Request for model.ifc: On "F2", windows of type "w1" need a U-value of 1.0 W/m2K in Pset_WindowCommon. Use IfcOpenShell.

First a look at what the model holds.

```python
import ifcopenshell
import ifcopenshell.util.element

model = ifcopenshell.open("model.ifc")
print(model.schema)
storey = next(s for s in model.by_type("IfcBuildingStorey") if s.Name == "F2")
windows = [e for e in ifcopenshell.util.element.get_decomposition(storey) if e.is_a("IfcWindow")]
seen = {}
for e in windows:
    element_type = ifcopenshell.util.element.get_type(e)
    key = (element_type.Name if element_type != e and element_type else None, ifcopenshell.util.element.get_pset(e, "Pset_WindowCommon", "ThermalTransmittance"))
    seen[key] = seen.get(key, 0) + 1
for (name, value), count in sorted(seen.items(), key=str):
    print(count, "x", name, "|", value)
```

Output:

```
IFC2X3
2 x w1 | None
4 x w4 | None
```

```python
import ifcopenshell
import ifcopenshell.api.pset
import ifcopenshell.util.element

model = ifcopenshell.open("model.ifc")

storey = next(s for s in model.by_type("IfcBuildingStorey") if s.Name == "F2")
windows = [e for e in ifcopenshell.util.element.get_decomposition(storey) if e.is_a("IfcWindow")]

count = 0
for e in windows:
    element_type = ifcopenshell.util.element.get_type(e)
    if element_type in (None, e) or element_type.Name != "w1":
        continue
    # add_pset returns the element's existing set when there is one.
    pset = ifcopenshell.api.pset.add_pset(model, product=e, name="Pset_WindowCommon")
    ifcopenshell.api.pset.edit_pset(model, pset=pset, properties={"ThermalTransmittance": 1.0})
    count += 1

print(count, "windows updated")

model.write("model_v2.ifc")
```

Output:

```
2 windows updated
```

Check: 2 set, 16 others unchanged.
